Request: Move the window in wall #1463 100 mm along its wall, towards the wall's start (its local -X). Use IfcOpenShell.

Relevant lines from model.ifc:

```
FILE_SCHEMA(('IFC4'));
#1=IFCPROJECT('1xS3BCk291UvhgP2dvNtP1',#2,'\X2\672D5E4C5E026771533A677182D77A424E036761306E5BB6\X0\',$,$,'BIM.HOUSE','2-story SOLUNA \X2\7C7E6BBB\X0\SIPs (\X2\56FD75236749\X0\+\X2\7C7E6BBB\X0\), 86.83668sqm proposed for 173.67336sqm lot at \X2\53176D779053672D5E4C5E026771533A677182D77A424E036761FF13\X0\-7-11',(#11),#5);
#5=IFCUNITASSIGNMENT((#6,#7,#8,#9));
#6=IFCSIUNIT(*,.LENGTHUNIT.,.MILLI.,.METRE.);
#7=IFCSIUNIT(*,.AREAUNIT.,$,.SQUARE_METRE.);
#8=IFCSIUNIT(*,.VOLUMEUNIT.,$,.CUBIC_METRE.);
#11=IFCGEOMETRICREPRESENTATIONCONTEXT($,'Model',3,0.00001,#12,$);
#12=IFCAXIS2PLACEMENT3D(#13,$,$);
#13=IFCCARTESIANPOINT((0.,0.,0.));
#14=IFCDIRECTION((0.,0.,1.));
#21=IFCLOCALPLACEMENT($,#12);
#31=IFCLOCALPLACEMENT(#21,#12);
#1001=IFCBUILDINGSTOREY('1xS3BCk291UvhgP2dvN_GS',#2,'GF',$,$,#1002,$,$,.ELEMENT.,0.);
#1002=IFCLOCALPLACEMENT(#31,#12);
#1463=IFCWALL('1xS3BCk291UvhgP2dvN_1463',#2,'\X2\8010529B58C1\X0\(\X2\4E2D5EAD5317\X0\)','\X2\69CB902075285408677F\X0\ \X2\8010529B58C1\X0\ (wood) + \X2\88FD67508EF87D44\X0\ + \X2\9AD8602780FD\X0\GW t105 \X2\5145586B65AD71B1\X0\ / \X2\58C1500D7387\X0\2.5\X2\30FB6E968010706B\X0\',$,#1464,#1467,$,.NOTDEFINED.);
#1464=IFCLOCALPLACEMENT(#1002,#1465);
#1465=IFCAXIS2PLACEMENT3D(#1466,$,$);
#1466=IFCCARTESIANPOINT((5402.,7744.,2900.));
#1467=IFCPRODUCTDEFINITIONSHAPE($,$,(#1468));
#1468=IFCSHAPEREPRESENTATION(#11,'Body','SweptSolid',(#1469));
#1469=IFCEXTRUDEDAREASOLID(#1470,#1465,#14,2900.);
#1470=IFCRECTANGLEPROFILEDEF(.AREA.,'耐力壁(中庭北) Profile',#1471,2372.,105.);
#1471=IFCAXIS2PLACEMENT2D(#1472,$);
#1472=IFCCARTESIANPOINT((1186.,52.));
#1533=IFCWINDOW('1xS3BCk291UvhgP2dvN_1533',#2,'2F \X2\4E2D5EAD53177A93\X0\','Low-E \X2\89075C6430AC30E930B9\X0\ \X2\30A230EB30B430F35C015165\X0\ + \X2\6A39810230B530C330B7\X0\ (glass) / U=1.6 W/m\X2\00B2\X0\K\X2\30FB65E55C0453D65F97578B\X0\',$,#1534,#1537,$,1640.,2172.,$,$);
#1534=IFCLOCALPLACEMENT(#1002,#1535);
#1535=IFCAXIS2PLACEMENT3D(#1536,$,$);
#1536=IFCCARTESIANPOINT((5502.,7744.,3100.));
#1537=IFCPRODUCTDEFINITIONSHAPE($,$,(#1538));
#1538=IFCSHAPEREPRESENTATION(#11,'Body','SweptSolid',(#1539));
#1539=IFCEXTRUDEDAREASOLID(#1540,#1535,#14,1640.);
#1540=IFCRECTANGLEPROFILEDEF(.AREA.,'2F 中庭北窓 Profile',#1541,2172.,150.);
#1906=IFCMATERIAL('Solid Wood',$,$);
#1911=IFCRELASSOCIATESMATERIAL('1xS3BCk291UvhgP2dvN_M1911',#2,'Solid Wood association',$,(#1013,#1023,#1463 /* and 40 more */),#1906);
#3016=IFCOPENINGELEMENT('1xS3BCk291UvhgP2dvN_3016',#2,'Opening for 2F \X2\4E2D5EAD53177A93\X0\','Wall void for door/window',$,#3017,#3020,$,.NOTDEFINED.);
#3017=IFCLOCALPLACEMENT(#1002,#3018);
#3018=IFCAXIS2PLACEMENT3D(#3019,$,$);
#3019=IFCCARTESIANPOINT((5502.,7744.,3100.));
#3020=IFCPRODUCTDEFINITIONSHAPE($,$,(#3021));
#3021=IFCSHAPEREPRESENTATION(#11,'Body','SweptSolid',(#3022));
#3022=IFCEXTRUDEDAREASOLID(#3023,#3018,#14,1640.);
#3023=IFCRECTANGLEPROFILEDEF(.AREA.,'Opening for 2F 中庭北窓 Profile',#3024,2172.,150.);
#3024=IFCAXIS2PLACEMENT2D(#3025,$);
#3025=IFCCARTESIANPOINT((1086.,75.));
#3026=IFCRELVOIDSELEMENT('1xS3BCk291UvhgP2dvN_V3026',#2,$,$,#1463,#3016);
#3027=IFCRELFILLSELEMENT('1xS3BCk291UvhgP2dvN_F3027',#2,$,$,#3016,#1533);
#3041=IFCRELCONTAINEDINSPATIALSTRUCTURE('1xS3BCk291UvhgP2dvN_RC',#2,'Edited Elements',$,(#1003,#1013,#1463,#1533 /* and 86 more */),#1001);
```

```python
import ifcopenshell
import ifcopenshell.api.geometry
import ifcopenshell.util.placement

model = ifcopenshell.open("model.ifc")

window = model.by_guid("1xS3BCk291UvhgP2dvN_1533")
opening = window.FillsVoids[0].RelatingOpeningElement
wall = opening.VoidsElements[0].RelatingBuildingElement

wall_matrix = ifcopenshell.util.placement.get_local_placement(wall.ObjectPlacement)
shift = wall_matrix[:3, 0] * -100.0
before = ifcopenshell.util.placement.get_local_placement(window.ObjectPlacement)[:3, 3].copy()

# The window is not placed relative to its opening, so move both.
for product in (opening, window):
    matrix = ifcopenshell.util.placement.get_local_placement(product.ObjectPlacement)
    matrix[:3, 3] += shift
    ifcopenshell.api.geometry.edit_object_placement(model, product=product, matrix=matrix, is_si=False)

after = ifcopenshell.util.placement.get_local_placement(window.ObjectPlacement)[:3, 3]
print("window moved by", (after - before).round(3) + 0.0)

model.write("model_updated.ifc")
```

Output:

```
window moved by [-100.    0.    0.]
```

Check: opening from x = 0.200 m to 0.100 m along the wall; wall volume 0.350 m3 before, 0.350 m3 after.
